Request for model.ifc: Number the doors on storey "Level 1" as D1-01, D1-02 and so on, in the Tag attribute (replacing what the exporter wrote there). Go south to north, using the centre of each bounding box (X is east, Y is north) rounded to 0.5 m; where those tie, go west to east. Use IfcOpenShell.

First a look at what the model holds.

```python
import ifcopenshell
import ifcopenshell.util.element
import ifcopenshell.util.placement

model = ifcopenshell.open("model.ifc")
print(model.schema)
storey = next(s for s in model.by_type("IfcBuildingStorey") if s.Name == "Level 1")
doors = [e for e in ifcopenshell.util.element.get_decomposition(storey) if e.is_a("IfcDoor")]
for e in sorted(doors, key=lambda e: e.id()):
    origin = ifcopenshell.util.placement.get_local_placement(e.ObjectPlacement)[:3, 3]
    print(e.id(), e.Tag, e.Name, origin.round(2) + 0.0, sep=" | ")
```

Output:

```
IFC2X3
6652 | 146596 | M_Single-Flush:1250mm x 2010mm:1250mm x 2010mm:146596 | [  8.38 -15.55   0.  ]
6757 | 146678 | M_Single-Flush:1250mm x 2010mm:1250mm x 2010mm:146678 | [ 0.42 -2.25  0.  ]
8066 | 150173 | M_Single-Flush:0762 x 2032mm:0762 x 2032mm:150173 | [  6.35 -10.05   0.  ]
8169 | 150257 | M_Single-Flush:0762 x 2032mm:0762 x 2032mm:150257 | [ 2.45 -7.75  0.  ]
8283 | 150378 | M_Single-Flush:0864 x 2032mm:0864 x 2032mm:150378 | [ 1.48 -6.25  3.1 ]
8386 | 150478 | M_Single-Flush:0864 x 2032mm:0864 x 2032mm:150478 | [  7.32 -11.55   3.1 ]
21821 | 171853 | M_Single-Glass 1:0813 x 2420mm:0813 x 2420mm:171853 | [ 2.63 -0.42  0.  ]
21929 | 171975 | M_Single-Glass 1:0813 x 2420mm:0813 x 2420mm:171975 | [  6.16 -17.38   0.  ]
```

```python
import ifcopenshell
import ifcopenshell.geom
import ifcopenshell.util.element
import ifcopenshell.util.shape

model = ifcopenshell.open("model.ifc")
settings = ifcopenshell.geom.settings()
settings.set("use-world-coords", True)


def centre(element):
    shape = ifcopenshell.geom.create_shape(settings, element)
    return ifcopenshell.util.shape.get_bbox_centroid(shape.geometry)


storey = next(s for s in model.by_type("IfcBuildingStorey") if s.Name == "Level 1")
doors = [e for e in ifcopenshell.util.element.get_decomposition(storey) if e.is_a("IfcDoor")]

# Insertion points can sit at a corner or the storey origin, so sort by the geometry (in metres).
centres = {e: centre(e) for e in doors}
doors.sort(key=lambda e: (round(centres[e][1] / 0.5), centres[e][0]))

for i, e in enumerate(doors, start=1):
    number = f"D1-{i:02d}"
    e.Tag = number
    print(e.id(), number)

model.write("model_v2.ifc")
```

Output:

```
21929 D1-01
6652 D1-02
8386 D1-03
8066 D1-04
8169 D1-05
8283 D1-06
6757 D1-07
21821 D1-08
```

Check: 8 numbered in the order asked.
